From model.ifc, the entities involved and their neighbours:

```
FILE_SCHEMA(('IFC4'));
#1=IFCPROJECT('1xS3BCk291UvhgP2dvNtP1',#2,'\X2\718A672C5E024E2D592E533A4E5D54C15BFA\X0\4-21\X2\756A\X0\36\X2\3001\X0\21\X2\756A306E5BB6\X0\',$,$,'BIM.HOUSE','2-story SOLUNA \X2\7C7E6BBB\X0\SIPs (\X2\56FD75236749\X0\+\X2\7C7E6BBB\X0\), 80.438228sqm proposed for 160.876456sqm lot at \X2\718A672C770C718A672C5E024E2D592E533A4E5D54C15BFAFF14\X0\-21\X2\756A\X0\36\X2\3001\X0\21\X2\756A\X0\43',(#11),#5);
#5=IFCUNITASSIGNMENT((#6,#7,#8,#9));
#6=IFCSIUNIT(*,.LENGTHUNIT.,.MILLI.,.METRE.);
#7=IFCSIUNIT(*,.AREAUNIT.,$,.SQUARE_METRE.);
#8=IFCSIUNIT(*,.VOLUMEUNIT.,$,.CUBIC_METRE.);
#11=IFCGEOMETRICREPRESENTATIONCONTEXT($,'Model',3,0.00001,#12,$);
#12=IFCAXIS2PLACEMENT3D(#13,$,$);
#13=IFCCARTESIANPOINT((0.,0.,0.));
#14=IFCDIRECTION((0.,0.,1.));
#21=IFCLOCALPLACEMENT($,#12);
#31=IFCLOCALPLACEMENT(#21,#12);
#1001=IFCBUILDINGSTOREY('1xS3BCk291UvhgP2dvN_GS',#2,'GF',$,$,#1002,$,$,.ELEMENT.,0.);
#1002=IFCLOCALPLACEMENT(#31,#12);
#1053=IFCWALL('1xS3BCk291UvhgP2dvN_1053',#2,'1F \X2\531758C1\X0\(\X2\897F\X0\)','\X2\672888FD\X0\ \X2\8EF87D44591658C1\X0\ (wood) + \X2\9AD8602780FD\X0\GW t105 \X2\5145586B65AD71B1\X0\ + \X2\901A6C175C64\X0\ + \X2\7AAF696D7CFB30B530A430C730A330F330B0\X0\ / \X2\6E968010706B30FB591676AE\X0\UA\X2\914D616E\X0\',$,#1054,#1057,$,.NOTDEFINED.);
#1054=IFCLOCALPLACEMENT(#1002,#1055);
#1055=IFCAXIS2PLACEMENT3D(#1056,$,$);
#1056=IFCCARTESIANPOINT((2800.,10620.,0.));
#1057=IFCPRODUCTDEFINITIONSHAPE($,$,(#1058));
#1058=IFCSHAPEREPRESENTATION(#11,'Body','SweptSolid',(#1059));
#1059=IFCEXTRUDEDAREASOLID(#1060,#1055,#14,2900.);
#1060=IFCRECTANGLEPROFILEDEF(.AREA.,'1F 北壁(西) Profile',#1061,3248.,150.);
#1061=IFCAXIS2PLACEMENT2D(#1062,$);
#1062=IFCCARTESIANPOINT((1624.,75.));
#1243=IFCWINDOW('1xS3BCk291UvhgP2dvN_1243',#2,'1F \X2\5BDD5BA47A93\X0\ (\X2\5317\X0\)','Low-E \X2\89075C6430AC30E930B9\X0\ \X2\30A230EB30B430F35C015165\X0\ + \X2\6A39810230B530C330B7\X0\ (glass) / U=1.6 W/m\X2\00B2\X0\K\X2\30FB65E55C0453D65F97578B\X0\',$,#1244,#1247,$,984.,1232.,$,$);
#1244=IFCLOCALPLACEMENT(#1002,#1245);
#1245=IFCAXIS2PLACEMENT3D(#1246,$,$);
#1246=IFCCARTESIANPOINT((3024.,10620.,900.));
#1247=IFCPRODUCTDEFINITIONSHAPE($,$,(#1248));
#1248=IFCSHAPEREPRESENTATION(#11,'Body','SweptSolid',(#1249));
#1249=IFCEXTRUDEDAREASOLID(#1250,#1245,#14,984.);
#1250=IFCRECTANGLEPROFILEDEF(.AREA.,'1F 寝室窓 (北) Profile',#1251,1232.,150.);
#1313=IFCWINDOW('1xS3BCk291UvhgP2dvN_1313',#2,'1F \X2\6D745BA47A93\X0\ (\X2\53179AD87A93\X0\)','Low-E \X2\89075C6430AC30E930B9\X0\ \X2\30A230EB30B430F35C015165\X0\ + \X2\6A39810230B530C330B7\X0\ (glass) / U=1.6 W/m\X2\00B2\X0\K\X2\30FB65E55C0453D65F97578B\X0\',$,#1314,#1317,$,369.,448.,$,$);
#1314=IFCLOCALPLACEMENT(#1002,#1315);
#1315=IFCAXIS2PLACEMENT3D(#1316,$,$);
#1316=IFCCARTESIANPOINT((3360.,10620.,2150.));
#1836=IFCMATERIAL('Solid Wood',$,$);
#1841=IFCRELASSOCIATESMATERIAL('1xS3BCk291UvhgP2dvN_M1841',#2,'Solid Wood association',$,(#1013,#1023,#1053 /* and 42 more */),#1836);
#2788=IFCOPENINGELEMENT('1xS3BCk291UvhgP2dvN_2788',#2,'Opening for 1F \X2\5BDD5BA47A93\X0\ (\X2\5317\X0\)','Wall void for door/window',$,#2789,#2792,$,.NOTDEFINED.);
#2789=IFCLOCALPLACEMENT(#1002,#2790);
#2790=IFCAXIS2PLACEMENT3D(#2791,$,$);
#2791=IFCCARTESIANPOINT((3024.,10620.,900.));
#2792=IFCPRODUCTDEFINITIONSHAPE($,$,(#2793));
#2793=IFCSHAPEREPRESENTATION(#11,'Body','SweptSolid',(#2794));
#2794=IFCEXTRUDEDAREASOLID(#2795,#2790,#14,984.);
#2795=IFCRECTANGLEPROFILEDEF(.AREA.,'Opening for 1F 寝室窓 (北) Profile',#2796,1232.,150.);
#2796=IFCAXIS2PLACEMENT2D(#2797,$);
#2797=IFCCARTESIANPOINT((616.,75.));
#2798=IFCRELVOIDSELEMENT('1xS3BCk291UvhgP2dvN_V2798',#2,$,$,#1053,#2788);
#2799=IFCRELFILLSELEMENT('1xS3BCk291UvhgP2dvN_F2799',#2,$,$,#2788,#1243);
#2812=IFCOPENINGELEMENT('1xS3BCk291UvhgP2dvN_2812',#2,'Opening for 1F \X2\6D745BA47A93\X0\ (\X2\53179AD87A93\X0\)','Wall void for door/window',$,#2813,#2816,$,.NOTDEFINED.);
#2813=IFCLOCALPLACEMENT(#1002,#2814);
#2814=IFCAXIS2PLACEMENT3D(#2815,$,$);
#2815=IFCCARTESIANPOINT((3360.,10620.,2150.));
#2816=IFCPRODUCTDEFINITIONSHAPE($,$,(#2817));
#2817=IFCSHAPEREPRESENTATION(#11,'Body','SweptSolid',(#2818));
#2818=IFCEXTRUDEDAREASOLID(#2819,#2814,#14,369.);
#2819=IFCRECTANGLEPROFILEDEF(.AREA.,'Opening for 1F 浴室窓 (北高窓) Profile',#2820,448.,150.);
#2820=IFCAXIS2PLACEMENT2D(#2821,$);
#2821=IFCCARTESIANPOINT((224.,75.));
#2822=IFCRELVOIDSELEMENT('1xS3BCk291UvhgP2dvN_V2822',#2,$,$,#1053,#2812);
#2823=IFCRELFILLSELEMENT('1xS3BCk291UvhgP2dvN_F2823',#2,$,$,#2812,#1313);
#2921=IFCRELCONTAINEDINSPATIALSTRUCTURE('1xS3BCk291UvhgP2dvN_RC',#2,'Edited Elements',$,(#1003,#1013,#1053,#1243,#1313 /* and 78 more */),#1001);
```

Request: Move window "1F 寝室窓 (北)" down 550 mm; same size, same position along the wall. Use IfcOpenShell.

```python
import numpy as np
import ifcopenshell
import ifcopenshell.api.geometry
import ifcopenshell.util.placement
import ifcopenshell.util.unit

model = ifcopenshell.open("model.ifc")
unit_scale = ifcopenshell.util.unit.calculate_unit_scale(model)

window = model.by_guid("1xS3BCk291UvhgP2dvN_1243")
opening = window.FillsVoids[0].RelatingOpeningElement
dz = -550.0

shift = np.array([0.0, 0.0, dz])
# The window is not placed relative to its opening, so move both.
for product in (opening, window):
    matrix = ifcopenshell.util.placement.get_local_placement(product.ObjectPlacement)
    matrix[:3, 3] += shift
    ifcopenshell.api.geometry.edit_object_placement(model, product=product, matrix=matrix, is_si=False)

print(f"moved by {dz * unit_scale:+.3f} m")

model.write("model-out.ifc")
```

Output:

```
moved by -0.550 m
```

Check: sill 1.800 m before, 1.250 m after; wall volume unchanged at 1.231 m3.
